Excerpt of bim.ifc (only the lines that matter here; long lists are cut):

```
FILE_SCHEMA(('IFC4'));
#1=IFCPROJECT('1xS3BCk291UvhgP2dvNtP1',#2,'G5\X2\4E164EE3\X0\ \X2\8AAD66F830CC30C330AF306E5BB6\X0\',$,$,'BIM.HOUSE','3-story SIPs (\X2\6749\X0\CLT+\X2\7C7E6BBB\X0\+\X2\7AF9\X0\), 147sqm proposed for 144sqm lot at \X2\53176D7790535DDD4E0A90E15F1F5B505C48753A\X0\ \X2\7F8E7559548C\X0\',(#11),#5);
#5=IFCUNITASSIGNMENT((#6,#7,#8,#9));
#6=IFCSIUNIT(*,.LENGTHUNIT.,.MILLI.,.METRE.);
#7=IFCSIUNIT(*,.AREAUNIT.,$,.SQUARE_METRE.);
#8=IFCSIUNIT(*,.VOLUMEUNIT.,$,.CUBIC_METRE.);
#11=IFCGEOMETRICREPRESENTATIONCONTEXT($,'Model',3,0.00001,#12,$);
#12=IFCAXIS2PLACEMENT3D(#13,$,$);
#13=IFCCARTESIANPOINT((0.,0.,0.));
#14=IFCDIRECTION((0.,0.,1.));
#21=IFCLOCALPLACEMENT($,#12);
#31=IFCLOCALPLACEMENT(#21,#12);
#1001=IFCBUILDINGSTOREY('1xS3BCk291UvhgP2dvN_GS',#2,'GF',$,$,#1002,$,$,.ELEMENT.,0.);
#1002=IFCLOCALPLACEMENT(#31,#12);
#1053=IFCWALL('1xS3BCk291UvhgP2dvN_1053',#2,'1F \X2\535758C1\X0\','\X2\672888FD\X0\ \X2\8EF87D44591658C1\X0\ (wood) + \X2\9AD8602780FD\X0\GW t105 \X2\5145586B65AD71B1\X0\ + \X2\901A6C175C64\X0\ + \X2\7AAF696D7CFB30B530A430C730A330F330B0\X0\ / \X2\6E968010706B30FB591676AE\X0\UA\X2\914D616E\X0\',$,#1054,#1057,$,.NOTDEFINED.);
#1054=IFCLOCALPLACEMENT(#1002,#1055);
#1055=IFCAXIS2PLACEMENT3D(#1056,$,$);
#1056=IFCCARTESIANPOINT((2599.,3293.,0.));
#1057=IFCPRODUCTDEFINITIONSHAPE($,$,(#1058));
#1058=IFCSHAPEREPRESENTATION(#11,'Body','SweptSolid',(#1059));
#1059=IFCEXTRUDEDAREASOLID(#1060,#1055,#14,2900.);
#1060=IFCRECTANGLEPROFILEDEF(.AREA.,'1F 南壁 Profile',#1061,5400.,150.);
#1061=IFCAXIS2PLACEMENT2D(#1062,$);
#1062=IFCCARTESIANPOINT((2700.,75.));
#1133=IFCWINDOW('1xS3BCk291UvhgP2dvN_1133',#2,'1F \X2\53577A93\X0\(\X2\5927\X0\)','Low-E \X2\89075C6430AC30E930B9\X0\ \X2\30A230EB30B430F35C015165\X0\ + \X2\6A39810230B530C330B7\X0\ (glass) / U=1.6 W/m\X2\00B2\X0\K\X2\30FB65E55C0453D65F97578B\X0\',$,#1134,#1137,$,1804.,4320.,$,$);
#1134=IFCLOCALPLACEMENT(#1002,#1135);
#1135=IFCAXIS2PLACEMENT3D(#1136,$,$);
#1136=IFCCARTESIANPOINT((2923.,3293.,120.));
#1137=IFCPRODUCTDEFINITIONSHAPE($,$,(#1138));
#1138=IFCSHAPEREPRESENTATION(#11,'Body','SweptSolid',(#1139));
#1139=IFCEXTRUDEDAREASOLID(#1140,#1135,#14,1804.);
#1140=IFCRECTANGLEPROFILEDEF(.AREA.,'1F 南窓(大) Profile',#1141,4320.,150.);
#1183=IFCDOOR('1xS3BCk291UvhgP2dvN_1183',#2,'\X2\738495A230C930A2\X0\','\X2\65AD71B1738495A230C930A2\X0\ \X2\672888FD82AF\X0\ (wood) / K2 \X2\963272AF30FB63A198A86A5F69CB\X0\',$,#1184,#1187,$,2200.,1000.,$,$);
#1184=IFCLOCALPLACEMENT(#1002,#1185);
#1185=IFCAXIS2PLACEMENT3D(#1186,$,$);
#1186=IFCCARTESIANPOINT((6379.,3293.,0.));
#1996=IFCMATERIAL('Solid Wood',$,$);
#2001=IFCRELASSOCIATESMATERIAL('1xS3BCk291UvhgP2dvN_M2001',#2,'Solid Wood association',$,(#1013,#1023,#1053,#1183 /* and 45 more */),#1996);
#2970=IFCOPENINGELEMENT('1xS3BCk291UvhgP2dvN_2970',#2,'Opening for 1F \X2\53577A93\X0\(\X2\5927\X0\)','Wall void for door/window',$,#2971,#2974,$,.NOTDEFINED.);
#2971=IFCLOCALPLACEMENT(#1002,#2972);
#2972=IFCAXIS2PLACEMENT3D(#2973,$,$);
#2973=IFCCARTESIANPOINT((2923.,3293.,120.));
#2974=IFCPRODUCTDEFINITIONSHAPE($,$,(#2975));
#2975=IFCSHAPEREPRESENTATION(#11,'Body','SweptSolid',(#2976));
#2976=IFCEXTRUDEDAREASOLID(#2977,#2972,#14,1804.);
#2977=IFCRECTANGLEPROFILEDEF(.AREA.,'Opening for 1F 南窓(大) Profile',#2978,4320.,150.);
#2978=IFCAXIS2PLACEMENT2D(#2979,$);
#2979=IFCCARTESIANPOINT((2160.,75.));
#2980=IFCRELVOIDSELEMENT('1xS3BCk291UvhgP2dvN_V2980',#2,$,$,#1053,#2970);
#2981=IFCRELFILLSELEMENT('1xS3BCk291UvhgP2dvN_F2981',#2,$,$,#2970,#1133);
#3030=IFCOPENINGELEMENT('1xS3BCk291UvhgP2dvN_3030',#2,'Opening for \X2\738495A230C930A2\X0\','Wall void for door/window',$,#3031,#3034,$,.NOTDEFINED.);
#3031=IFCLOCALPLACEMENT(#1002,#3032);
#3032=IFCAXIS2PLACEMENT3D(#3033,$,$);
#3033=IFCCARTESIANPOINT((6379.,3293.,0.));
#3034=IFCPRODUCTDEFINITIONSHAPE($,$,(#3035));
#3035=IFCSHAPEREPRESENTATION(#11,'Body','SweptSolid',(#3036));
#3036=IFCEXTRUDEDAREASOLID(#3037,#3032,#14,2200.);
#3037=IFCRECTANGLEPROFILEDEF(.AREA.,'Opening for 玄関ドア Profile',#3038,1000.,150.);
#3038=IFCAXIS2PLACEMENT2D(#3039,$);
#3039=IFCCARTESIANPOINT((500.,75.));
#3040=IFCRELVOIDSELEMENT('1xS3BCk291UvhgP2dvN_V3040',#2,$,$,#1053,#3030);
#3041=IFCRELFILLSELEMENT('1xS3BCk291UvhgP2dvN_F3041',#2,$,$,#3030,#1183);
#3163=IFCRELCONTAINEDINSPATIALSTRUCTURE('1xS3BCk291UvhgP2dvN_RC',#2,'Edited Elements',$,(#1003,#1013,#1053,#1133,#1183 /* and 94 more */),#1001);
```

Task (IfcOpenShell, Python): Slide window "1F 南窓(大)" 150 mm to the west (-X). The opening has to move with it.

```python
import ifcopenshell
import ifcopenshell.api.geometry
import ifcopenshell.util.placement
import ifcopenshell.util.unit

model = ifcopenshell.open("bim.ifc")
unit_scale = ifcopenshell.util.unit.calculate_unit_scale(model)

window = model.by_guid("1xS3BCk291UvhgP2dvN_1133")
opening = window.FillsVoids[0].RelatingOpeningElement
wall = opening.VoidsElements[0].RelatingBuildingElement

wall_matrix = ifcopenshell.util.placement.get_local_placement(wall.ObjectPlacement)
shift = wall_matrix[:3, 0] * -0.15 / unit_scale
before = ifcopenshell.util.placement.get_local_placement(window.ObjectPlacement)[:3, 3].copy()

# The window is not placed relative to its opening, so move both.
for product in (opening, window):
    matrix = ifcopenshell.util.placement.get_local_placement(product.ObjectPlacement)
    matrix[:3, 3] += shift
    ifcopenshell.api.geometry.edit_object_placement(model, product=product, matrix=matrix, is_si=False)

after = ifcopenshell.util.placement.get_local_placement(window.ObjectPlacement)[:3, 3]
print("window moved by", (after - before).round(3) + 0.0)

model.write("bim_rev.ifc")
```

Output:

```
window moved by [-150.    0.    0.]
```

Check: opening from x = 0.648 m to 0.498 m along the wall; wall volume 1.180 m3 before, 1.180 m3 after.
